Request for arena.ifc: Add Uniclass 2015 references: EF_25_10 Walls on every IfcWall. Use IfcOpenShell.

First a look at what the model holds.

```python
import ifcopenshell

model = ifcopenshell.open("arena.ifc")
print(model.schema)
print("classifications:", [c.Name for c in model.by_type("IfcClassification")])
for ifc_class in ("IfcDoor", "IfcRoof", "IfcStair", "IfcWall", "IfcWindow"):
    print(ifc_class, len(model.by_type(ifc_class)))
```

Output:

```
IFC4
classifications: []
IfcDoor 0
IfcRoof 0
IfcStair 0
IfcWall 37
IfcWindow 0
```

```python
import ifcopenshell
import ifcopenshell.api.classification

model = ifcopenshell.open("arena.ifc")

system = ifcopenshell.api.classification.add_classification(model, classification="Uniclass 2015")

codes = {
    "IfcWall": ("EF_25_10", "Walls"),
}
for ifc_class, (code, name) in codes.items():
    products = model.by_type(ifc_class)
    ifcopenshell.api.classification.add_reference(
        model, products=products, classification=system, identification=code, name=name
    )
    print(code, len(products))

model.write("arena_v2.ifc")
```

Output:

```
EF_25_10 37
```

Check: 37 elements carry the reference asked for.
